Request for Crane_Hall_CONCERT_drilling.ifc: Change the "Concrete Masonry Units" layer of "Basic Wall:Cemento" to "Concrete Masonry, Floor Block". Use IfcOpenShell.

First a look at what the model holds.

```python
import ifcopenshell
import ifcopenshell.util.element

model = ifcopenshell.open("Crane_Hall_CONCERT_drilling.ifc")
print(model.schema)
for layer_set in model.by_type("IfcMaterialLayerSet"):
    if layer_set.LayerSetName == "Basic Wall:Cemento":
        for layer in layer_set.MaterialLayers:
            print(layer.id(), layer.Material and layer.Material.Name, layer.LayerThickness, sep=" | ")
        print(len(ifcopenshell.util.element.get_elements_by_material(model, layer_set)), "elements and types use it")
print(sorted(m.Name for m in model.by_type("IfcMaterial") if m.Name)[:60])
```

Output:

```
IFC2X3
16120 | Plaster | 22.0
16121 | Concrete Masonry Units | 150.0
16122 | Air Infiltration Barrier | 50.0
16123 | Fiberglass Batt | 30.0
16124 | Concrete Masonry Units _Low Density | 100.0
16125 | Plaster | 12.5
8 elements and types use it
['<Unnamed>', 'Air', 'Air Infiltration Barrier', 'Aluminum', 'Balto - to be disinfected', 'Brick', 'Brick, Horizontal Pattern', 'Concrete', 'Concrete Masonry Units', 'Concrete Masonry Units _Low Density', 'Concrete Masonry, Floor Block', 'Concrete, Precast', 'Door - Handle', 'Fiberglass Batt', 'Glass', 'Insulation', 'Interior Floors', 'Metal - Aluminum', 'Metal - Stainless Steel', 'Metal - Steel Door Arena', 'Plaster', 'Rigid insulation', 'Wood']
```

```python
import ifcopenshell
import ifcopenshell.api.material

model = ifcopenshell.open("Crane_Hall_CONCERT_drilling.ifc")

layer_set = next(s for s in model.by_type("IfcMaterialLayerSet") if s.LayerSetName == "Basic Wall:Cemento")
layer = next(l for l in layer_set.MaterialLayers if l.Material and l.Material.Name == "Concrete Masonry Units")
material = next(m for m in model.by_type("IfcMaterial") if m.Name == "Concrete Masonry, Floor Block")

# Point this one layer at the other material; renaming the old one would change it everywhere.
ifcopenshell.api.material.edit_layer(model, layer=layer, attributes={}, material=material)

print([l.Material.Name if l.Material else None for l in layer_set.MaterialLayers])

model.write("Crane_Hall_CONCERT_drilling_v2.ifc")
```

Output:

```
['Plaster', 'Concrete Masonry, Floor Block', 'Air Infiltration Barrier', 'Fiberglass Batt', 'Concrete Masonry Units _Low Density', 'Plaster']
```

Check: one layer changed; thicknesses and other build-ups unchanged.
